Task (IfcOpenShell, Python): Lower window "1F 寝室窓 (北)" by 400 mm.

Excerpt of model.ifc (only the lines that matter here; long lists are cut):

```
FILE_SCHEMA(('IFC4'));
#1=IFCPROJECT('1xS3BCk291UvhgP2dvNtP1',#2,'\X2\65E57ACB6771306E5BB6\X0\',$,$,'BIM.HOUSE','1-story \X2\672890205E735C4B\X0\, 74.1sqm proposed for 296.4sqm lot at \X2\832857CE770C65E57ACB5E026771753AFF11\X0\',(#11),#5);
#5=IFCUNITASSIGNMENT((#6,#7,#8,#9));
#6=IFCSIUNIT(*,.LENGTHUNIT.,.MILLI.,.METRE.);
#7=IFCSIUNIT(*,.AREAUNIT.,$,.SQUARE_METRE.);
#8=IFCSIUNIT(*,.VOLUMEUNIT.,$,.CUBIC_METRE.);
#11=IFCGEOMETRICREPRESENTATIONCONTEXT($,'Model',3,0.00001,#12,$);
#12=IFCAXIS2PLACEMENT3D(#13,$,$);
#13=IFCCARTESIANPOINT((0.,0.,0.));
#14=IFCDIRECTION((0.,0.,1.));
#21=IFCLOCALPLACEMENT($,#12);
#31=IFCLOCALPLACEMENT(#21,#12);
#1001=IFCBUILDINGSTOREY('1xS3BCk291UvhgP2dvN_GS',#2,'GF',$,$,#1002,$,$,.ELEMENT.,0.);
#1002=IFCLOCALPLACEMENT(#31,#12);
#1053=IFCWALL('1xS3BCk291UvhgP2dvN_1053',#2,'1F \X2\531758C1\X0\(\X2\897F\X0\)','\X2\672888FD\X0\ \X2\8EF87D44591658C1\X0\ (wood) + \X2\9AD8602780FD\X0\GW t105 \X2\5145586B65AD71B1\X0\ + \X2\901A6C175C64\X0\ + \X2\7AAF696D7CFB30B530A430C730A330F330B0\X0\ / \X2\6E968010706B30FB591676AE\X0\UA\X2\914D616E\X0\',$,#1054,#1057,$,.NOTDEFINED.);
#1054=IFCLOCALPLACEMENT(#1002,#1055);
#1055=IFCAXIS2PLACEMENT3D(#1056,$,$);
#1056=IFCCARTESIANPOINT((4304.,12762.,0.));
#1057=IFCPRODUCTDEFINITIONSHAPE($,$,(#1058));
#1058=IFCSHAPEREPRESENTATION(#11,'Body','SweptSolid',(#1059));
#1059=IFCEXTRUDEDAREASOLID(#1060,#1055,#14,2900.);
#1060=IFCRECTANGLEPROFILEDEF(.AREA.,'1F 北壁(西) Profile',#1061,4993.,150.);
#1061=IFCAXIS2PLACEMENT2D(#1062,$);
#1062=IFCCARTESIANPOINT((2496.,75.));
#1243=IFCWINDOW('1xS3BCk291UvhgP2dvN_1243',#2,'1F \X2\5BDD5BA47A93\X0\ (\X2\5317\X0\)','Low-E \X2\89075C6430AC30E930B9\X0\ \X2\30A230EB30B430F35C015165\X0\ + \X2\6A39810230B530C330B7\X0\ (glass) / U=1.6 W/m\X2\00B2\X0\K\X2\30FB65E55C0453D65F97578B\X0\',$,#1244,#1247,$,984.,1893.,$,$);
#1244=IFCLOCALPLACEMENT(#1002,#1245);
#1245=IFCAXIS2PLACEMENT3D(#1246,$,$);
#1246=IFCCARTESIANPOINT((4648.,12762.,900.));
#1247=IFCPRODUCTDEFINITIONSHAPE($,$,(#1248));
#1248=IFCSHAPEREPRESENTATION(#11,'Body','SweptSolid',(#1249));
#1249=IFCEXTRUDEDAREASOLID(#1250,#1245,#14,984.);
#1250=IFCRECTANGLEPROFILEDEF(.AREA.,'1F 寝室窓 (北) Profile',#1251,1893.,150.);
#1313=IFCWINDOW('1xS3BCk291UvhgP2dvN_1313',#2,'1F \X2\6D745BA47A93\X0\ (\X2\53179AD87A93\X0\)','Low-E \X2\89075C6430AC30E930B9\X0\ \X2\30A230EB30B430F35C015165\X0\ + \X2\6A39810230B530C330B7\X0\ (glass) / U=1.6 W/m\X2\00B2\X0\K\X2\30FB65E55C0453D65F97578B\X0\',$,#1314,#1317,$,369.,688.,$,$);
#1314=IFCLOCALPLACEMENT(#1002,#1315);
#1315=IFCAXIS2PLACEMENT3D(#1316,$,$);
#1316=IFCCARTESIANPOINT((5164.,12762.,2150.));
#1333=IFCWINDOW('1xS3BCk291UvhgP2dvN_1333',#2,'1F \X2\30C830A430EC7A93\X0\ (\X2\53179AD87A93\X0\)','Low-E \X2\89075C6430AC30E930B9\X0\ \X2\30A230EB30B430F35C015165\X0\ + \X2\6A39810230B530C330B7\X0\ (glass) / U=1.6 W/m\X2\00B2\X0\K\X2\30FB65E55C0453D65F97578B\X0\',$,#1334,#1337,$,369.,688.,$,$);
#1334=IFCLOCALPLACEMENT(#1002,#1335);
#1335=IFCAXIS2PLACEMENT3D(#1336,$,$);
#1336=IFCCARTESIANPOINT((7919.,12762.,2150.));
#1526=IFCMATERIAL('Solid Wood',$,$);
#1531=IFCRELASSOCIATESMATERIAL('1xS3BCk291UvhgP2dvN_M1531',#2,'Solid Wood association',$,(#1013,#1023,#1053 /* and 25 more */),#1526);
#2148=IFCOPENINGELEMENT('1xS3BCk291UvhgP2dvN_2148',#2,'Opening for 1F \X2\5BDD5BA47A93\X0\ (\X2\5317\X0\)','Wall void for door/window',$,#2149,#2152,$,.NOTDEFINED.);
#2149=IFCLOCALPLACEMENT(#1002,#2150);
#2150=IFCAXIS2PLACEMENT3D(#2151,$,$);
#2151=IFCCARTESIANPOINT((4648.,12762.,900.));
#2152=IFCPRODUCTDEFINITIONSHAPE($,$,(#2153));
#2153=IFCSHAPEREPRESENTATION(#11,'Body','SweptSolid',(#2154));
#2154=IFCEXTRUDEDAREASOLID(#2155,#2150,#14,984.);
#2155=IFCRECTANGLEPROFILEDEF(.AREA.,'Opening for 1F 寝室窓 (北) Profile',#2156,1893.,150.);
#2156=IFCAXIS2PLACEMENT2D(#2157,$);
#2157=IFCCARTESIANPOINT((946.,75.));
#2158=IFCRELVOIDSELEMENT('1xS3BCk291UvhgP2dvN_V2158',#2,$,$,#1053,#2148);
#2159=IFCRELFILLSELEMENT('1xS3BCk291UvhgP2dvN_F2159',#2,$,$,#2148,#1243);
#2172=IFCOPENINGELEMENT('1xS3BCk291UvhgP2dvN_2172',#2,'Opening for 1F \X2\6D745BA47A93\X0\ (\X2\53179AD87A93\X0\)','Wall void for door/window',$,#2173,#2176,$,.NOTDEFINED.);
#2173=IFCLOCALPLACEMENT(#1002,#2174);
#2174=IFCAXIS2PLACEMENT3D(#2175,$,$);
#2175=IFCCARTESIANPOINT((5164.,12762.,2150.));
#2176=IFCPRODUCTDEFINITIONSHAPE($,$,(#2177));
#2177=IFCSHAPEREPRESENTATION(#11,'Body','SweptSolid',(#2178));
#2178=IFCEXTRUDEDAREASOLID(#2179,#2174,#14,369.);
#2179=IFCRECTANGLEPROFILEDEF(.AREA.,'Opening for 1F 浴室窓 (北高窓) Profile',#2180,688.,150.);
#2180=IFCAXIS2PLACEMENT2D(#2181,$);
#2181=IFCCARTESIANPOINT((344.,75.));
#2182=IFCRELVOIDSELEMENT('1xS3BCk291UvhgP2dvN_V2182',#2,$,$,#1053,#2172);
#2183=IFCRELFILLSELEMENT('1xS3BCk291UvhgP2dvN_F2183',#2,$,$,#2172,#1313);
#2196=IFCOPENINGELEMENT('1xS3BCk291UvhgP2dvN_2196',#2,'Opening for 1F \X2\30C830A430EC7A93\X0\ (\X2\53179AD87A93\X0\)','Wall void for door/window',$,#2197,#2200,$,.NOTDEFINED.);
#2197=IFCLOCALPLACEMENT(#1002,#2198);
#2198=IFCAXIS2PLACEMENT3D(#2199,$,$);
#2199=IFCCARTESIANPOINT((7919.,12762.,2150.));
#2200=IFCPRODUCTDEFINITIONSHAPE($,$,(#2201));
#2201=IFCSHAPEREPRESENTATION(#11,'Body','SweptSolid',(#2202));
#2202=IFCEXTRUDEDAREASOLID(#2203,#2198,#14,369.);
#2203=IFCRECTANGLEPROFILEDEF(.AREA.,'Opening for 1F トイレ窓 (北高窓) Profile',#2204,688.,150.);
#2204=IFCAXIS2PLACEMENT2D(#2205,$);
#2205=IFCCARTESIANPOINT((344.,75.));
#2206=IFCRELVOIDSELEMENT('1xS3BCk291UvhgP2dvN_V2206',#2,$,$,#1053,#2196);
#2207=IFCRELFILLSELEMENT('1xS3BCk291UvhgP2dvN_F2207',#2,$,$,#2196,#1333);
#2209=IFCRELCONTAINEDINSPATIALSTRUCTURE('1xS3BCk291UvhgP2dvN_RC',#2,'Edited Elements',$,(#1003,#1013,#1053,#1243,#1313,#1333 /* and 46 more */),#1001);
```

```python
import numpy as np
import ifcopenshell
import ifcopenshell.api.geometry
import ifcopenshell.util.placement
import ifcopenshell.util.unit

model = ifcopenshell.open("model.ifc")
unit_scale = ifcopenshell.util.unit.calculate_unit_scale(model)

window = model.by_id(1243)
opening = window.FillsVoids[0].RelatingOpeningElement
dz = -400.0

shift = np.array([0.0, 0.0, dz])
# The window is not placed relative to its opening, so move both.
for product in (opening, window):
    matrix = ifcopenshell.util.placement.get_local_placement(product.ObjectPlacement)
    matrix[:3, 3] += shift
    ifcopenshell.api.geometry.edit_object_placement(model, product=product, matrix=matrix, is_si=False)

print(f"moved by {dz * unit_scale:+.3f} m")

model.write("model_updated.ifc")
```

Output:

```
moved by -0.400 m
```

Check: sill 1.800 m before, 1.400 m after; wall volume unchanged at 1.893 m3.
